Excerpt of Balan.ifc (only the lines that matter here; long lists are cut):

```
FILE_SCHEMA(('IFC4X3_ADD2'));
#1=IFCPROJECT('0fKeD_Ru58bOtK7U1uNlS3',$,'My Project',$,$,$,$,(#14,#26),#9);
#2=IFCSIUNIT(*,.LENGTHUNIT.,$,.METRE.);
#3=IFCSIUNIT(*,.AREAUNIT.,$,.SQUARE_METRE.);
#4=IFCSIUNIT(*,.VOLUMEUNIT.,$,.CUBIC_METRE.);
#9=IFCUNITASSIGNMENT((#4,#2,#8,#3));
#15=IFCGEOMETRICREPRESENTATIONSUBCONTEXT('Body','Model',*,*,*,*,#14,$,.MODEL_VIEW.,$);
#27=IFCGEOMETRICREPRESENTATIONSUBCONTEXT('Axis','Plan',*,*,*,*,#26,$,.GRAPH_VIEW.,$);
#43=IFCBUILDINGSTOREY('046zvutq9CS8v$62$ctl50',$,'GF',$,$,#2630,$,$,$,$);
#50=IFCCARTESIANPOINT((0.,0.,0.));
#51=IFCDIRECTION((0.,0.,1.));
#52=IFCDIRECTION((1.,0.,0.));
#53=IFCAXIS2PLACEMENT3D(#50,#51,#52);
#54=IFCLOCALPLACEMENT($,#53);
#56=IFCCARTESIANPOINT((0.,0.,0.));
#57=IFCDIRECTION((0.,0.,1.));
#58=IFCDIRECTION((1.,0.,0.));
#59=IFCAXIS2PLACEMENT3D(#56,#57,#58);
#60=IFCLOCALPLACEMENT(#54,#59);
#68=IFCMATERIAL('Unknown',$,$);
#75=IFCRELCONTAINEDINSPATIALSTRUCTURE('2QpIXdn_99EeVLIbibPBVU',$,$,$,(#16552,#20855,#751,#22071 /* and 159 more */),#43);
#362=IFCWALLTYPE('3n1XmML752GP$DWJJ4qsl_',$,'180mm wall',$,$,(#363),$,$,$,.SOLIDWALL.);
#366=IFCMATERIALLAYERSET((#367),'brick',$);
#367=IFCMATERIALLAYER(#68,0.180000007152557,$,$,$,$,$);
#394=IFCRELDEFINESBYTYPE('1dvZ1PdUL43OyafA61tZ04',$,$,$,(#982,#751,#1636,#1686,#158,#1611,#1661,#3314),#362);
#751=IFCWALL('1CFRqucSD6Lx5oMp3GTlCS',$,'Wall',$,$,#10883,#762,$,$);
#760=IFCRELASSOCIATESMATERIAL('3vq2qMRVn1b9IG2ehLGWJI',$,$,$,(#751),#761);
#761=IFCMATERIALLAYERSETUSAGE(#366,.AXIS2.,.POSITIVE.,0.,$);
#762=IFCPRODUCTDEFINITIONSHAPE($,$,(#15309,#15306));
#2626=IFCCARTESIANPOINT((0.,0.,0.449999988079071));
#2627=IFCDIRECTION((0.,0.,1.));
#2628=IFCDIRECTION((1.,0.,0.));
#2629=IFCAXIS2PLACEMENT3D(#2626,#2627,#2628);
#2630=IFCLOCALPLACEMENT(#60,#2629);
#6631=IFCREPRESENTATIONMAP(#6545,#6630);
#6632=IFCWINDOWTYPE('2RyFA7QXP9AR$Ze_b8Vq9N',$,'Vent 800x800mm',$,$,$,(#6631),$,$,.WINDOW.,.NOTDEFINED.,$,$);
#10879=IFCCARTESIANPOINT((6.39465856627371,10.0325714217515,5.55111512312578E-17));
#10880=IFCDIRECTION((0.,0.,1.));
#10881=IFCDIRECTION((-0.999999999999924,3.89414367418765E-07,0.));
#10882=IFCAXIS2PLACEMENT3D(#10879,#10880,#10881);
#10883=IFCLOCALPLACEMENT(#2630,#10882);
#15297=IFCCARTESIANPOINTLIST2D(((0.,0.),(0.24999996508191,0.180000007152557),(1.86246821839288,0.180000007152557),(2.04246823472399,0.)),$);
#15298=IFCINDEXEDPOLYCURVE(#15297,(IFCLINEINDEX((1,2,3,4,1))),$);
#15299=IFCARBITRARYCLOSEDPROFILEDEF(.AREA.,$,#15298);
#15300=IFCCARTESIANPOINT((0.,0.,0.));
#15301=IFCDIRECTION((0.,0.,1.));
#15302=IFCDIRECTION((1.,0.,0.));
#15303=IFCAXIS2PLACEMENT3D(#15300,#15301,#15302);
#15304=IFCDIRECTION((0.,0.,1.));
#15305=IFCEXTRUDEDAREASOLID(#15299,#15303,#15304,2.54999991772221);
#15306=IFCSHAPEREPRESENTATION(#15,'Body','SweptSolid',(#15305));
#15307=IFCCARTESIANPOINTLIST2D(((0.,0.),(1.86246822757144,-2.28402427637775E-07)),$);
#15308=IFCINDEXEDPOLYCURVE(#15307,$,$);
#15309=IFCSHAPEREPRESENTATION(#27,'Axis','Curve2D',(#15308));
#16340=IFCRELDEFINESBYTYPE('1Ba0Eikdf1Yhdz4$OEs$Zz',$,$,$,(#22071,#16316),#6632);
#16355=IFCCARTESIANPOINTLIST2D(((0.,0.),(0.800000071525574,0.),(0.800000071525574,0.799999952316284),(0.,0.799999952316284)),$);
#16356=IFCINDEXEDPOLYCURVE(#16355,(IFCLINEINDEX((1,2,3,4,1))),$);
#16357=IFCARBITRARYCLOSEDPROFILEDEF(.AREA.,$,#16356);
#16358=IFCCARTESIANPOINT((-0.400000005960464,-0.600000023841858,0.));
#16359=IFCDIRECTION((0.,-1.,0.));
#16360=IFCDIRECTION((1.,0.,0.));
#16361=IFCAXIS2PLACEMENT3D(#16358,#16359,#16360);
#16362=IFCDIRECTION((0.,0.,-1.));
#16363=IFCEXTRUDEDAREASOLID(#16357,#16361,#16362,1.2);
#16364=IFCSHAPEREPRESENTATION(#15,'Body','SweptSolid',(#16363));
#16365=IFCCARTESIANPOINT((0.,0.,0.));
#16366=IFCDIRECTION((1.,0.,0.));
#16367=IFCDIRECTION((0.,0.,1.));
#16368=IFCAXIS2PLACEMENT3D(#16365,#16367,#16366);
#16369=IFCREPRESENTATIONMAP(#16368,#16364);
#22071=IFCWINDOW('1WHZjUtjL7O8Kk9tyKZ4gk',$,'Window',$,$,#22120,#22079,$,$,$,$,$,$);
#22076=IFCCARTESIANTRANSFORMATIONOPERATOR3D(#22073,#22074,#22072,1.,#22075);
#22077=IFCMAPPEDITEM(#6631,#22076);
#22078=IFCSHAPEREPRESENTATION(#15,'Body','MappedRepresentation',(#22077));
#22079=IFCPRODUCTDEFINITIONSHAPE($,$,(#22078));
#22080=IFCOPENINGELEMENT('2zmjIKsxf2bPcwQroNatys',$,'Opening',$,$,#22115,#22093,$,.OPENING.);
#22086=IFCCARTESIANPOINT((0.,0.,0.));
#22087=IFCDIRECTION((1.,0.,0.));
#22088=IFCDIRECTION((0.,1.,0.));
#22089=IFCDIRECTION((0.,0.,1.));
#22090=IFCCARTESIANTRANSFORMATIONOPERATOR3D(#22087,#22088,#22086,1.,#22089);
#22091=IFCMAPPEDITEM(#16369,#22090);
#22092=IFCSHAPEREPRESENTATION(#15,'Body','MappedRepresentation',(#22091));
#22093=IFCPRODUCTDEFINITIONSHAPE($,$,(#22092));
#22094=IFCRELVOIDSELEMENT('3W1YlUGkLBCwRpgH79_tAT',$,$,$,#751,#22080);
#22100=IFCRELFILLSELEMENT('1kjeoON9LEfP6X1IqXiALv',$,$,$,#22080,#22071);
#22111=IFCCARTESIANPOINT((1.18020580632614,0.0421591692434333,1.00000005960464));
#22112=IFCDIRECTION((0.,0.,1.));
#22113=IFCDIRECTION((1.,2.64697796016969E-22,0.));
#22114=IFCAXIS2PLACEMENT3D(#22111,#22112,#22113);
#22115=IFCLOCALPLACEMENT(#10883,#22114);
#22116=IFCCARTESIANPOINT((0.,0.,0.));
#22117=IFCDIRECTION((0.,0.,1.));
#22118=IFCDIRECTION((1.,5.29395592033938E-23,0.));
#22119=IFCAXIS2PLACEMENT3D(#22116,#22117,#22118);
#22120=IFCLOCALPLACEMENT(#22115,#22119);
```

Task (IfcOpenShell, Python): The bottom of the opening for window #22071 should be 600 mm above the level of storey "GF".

```python
import numpy as np
import ifcopenshell
import ifcopenshell.api.geometry
import ifcopenshell.geom
import ifcopenshell.util.element
import ifcopenshell.util.placement
import ifcopenshell.util.shape
import ifcopenshell.util.unit

model = ifcopenshell.open("Balan.ifc")
unit_scale = ifcopenshell.util.unit.calculate_unit_scale(model)

window = model.by_guid("1WHZjUtjL7O8Kk9tyKZ4gk")
opening = window.FillsVoids[0].RelatingOpeningElement
storey = ifcopenshell.util.element.get_container(window, ifc_class="IfcBuildingStorey")
level = ifcopenshell.util.placement.get_local_placement(storey.ObjectPlacement)[2, 3]

# The opening's origin need not be at the sill, so measure its lowest point.
shape = ifcopenshell.geom.create_shape(ifcopenshell.geom.settings(), opening)
bottom = ifcopenshell.util.shape.get_shape_bottom_elevation(shape, shape.geometry) / unit_scale
dz = level + 0.6 / unit_scale - bottom

shift = np.array([0.0, 0.0, dz])
# The window is placed relative to its opening, so it follows when the opening moves.
matrix = ifcopenshell.util.placement.get_local_placement(opening.ObjectPlacement)
matrix[:3, 3] += shift
ifcopenshell.api.geometry.edit_object_placement(
    model, product=opening, matrix=matrix, is_si=False, should_transform_children=True
)

print(f"moved by {dz * unit_scale:+.3f} m")

model.write("Balan_v2.ifc")
```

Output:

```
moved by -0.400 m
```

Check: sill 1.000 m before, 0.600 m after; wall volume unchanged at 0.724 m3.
